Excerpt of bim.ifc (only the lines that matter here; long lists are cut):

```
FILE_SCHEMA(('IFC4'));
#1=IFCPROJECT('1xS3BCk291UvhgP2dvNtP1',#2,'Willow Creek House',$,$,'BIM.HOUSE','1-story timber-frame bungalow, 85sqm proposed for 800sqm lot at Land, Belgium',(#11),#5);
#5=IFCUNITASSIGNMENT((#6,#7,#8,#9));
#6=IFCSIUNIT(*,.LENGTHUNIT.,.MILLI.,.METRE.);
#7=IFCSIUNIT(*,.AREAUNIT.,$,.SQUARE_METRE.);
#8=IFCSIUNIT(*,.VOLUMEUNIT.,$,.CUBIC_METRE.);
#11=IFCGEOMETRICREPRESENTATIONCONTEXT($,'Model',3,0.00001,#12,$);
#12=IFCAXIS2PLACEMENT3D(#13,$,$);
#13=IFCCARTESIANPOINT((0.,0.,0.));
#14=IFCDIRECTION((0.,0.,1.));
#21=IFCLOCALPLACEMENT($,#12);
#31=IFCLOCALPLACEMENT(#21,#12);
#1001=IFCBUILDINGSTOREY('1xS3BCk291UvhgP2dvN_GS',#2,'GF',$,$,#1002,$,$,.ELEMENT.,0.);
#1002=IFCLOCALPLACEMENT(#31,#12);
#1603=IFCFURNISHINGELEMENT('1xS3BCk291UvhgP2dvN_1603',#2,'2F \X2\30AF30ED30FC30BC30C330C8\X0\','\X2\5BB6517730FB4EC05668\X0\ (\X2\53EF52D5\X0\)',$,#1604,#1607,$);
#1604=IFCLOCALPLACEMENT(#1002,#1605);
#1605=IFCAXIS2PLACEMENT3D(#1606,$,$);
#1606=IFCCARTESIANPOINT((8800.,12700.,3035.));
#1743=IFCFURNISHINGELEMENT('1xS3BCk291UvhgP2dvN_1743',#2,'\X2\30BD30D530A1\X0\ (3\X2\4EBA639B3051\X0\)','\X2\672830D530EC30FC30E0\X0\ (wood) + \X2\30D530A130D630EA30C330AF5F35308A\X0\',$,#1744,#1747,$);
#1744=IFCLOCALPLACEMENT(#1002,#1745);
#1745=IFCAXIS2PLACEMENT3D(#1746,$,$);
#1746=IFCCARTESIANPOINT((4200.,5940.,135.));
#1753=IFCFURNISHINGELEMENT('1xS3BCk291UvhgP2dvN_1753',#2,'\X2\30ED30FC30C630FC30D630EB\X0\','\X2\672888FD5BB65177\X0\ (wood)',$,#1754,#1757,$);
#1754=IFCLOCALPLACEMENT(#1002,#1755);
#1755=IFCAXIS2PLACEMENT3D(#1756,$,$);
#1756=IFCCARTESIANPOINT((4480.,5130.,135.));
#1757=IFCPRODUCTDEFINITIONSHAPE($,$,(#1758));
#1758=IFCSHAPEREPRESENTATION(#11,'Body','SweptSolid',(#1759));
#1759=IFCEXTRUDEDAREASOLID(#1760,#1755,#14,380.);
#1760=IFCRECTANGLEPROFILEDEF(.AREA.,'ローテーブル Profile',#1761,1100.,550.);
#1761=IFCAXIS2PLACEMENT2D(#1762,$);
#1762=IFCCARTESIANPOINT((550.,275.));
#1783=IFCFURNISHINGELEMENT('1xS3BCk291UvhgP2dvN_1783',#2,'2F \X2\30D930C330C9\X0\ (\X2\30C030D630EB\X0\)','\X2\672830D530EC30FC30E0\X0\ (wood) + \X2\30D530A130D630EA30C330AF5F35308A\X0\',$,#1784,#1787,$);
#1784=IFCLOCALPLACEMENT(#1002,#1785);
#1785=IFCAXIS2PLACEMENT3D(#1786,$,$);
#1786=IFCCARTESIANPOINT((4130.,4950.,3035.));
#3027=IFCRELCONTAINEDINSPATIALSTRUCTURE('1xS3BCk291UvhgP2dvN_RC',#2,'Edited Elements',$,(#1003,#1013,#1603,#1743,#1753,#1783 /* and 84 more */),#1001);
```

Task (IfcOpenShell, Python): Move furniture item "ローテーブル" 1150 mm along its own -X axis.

```python
import ifcopenshell
import ifcopenshell.api.geometry
import ifcopenshell.util.placement
import ifcopenshell.util.unit

model = ifcopenshell.open("bim.ifc")
unit_scale = ifcopenshell.util.unit.calculate_unit_scale(model)

item = model.by_guid("1xS3BCk291UvhgP2dvN_1753")
matrix = ifcopenshell.util.placement.get_local_placement(item.ObjectPlacement)
matrix[:3, 3] -= matrix[:3, 0] * 1.15 / unit_scale
ifcopenshell.api.geometry.edit_object_placement(model, product=item, matrix=matrix, is_si=False)

print(ifcopenshell.util.placement.get_local_placement(item.ObjectPlacement).round(3) + 0.0)

model.write("bim_rev.ifc")
```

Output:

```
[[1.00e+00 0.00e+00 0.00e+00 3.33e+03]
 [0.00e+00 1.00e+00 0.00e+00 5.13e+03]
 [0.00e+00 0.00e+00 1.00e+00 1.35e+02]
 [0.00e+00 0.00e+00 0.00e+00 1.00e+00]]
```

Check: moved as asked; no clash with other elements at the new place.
